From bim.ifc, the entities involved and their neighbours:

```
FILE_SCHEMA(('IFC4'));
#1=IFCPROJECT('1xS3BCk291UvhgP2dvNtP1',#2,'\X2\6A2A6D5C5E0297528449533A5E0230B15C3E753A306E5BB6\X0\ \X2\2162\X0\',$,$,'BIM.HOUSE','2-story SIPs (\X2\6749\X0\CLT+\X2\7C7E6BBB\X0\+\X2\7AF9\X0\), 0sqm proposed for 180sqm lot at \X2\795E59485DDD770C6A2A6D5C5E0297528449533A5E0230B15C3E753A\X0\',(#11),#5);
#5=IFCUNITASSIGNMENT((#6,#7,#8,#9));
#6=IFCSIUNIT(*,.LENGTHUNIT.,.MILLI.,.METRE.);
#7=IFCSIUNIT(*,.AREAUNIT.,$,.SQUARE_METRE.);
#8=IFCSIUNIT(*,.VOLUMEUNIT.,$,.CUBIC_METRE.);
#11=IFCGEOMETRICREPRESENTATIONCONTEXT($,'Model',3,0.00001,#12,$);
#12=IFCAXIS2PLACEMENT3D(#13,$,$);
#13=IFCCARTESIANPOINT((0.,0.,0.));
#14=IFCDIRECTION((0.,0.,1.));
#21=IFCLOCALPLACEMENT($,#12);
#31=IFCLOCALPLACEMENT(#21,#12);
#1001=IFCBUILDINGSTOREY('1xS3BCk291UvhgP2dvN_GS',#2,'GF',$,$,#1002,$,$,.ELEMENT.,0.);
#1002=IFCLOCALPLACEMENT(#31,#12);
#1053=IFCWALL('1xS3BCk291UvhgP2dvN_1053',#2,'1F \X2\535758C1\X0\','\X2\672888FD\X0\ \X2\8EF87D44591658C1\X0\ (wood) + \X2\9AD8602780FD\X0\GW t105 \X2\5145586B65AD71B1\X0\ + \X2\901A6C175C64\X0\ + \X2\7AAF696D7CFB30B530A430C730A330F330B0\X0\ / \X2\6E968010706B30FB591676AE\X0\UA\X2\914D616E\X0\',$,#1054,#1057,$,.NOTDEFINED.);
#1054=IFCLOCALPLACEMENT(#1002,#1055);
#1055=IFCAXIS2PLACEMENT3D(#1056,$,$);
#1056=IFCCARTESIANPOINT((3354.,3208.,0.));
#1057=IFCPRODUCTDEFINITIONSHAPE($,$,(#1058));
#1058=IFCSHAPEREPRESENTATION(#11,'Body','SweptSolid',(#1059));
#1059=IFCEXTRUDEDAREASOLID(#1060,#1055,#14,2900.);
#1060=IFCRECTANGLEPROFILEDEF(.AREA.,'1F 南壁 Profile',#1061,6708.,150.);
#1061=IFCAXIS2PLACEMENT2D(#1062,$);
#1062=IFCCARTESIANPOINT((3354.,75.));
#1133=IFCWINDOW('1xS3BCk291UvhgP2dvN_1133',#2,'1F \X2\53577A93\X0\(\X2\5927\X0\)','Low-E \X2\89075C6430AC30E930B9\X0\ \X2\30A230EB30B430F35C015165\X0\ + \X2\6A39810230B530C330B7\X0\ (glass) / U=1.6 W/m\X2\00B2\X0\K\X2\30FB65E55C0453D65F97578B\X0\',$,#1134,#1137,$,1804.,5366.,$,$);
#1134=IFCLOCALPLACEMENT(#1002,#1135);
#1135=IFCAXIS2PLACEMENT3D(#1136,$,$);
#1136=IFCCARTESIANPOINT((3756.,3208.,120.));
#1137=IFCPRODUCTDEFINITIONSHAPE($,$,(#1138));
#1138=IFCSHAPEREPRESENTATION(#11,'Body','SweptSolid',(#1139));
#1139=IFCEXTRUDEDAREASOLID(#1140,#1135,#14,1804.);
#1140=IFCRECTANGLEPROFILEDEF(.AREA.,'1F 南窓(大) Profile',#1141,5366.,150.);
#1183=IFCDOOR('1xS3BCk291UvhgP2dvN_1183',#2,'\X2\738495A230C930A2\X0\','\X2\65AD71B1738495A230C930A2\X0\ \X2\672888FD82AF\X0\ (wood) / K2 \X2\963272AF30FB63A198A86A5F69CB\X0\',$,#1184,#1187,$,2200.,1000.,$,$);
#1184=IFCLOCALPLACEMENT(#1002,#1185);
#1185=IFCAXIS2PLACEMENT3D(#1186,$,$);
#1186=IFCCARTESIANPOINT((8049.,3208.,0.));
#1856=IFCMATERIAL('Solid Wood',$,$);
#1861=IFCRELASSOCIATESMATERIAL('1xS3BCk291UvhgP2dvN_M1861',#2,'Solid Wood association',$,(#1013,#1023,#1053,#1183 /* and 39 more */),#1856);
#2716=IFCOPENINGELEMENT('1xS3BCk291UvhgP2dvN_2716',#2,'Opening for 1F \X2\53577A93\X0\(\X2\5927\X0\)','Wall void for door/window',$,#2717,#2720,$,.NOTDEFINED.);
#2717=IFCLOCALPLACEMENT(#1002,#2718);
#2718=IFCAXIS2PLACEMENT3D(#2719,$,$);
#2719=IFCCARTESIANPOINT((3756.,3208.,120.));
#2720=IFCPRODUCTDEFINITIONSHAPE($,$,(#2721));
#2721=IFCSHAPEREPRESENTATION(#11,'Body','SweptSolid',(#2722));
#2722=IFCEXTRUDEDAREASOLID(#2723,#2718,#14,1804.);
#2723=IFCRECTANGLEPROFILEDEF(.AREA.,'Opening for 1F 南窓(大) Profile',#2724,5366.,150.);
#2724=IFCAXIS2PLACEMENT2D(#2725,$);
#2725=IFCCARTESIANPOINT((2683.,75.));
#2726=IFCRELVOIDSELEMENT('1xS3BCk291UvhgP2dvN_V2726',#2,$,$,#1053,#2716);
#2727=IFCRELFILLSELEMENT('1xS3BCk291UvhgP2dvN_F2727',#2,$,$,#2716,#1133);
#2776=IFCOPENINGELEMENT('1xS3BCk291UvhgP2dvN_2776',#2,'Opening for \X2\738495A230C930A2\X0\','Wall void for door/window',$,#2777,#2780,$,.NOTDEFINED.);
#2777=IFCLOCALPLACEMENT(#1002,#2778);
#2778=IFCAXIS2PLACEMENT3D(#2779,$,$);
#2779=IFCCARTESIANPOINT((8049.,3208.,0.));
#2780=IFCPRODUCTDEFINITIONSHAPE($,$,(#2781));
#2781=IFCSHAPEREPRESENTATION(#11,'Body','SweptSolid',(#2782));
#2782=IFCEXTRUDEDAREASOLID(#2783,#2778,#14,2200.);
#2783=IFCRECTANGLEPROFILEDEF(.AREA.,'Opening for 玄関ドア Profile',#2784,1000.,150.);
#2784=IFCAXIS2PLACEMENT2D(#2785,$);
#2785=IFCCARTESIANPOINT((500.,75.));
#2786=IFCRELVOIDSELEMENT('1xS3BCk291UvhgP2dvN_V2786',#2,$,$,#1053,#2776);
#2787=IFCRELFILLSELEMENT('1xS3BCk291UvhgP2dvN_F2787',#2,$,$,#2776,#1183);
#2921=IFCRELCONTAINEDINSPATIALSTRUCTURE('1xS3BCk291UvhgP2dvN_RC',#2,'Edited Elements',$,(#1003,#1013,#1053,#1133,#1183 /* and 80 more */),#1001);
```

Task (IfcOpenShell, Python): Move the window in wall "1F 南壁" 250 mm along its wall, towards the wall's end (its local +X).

```python
import ifcopenshell
import ifcopenshell.api.geometry
import ifcopenshell.util.placement
import ifcopenshell.util.unit

model = ifcopenshell.open("bim.ifc")
unit_scale = ifcopenshell.util.unit.calculate_unit_scale(model)

window = model.by_guid("1xS3BCk291UvhgP2dvN_1133")
opening = window.FillsVoids[0].RelatingOpeningElement
wall = opening.VoidsElements[0].RelatingBuildingElement

wall_matrix = ifcopenshell.util.placement.get_local_placement(wall.ObjectPlacement)
shift = wall_matrix[:3, 0] * 0.25 / unit_scale
before = ifcopenshell.util.placement.get_local_placement(window.ObjectPlacement)[:3, 3].copy()

# The window is not placed relative to its opening, so move both.
for product in (opening, window):
    matrix = ifcopenshell.util.placement.get_local_placement(product.ObjectPlacement)
    matrix[:3, 3] += shift
    ifcopenshell.api.geometry.edit_object_placement(model, product=product, matrix=matrix, is_si=False)

after = ifcopenshell.util.placement.get_local_placement(window.ObjectPlacement)[:3, 3]
print("window moved by", (after - before).round(3) + 0.0)

model.write("bim-out.ifc")
```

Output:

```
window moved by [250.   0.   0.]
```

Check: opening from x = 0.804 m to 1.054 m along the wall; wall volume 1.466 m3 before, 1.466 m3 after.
